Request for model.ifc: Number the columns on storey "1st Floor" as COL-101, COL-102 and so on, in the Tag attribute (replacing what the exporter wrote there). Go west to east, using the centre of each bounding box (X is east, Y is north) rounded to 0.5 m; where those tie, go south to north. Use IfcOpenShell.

First a look at what the model holds.

```python
import ifcopenshell
import ifcopenshell.util.element
import ifcopenshell.util.placement

model = ifcopenshell.open("model.ifc")
print(model.schema)
storey = next(s for s in model.by_type("IfcBuildingStorey") if s.Name == "1st Floor")
columns = [e for e in ifcopenshell.util.element.get_decomposition(storey) if e.is_a("IfcColumn")]
for e in sorted(columns, key=lambda e: e.id()):
    origin = ifcopenshell.util.placement.get_local_placement(e.ObjectPlacement)[:3, 3]
    print(e.id(), e.Tag, e.Name, origin.round(2) + 0.0, sep=" | ")
```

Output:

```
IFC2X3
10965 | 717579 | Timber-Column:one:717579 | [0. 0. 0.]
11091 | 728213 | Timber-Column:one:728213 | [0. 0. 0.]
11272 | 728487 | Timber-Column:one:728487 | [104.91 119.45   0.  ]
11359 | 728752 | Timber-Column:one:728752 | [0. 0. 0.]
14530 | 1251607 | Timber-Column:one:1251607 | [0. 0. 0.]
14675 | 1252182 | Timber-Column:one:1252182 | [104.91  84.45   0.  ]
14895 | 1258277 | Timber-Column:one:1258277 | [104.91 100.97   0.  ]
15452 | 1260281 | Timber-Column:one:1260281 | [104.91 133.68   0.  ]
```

```python
import ifcopenshell
import ifcopenshell.geom
import ifcopenshell.util.element
import ifcopenshell.util.shape

model = ifcopenshell.open("model.ifc")
settings = ifcopenshell.geom.settings()
settings.set("use-world-coords", True)


def centre(element):
    shape = ifcopenshell.geom.create_shape(settings, element)
    return ifcopenshell.util.shape.get_bbox_centroid(shape.geometry)


storey = next(s for s in model.by_type("IfcBuildingStorey") if s.Name == "1st Floor")
columns = [e for e in ifcopenshell.util.element.get_decomposition(storey) if e.is_a("IfcColumn")]

# Insertion points can sit at a corner or the storey origin, so sort by the geometry (in metres).
centres = {e: centre(e) for e in columns}
columns.sort(key=lambda e: (round(centres[e][0] / 0.5), centres[e][1]))

for i, e in enumerate(columns, start=1):
    number = f"COL-1{i:02d}"
    e.Tag = number
    print(e.id(), number)

model.write("model_updated.ifc")
```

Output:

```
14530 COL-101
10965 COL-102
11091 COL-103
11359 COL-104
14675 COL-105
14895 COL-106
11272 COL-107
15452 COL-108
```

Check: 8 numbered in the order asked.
